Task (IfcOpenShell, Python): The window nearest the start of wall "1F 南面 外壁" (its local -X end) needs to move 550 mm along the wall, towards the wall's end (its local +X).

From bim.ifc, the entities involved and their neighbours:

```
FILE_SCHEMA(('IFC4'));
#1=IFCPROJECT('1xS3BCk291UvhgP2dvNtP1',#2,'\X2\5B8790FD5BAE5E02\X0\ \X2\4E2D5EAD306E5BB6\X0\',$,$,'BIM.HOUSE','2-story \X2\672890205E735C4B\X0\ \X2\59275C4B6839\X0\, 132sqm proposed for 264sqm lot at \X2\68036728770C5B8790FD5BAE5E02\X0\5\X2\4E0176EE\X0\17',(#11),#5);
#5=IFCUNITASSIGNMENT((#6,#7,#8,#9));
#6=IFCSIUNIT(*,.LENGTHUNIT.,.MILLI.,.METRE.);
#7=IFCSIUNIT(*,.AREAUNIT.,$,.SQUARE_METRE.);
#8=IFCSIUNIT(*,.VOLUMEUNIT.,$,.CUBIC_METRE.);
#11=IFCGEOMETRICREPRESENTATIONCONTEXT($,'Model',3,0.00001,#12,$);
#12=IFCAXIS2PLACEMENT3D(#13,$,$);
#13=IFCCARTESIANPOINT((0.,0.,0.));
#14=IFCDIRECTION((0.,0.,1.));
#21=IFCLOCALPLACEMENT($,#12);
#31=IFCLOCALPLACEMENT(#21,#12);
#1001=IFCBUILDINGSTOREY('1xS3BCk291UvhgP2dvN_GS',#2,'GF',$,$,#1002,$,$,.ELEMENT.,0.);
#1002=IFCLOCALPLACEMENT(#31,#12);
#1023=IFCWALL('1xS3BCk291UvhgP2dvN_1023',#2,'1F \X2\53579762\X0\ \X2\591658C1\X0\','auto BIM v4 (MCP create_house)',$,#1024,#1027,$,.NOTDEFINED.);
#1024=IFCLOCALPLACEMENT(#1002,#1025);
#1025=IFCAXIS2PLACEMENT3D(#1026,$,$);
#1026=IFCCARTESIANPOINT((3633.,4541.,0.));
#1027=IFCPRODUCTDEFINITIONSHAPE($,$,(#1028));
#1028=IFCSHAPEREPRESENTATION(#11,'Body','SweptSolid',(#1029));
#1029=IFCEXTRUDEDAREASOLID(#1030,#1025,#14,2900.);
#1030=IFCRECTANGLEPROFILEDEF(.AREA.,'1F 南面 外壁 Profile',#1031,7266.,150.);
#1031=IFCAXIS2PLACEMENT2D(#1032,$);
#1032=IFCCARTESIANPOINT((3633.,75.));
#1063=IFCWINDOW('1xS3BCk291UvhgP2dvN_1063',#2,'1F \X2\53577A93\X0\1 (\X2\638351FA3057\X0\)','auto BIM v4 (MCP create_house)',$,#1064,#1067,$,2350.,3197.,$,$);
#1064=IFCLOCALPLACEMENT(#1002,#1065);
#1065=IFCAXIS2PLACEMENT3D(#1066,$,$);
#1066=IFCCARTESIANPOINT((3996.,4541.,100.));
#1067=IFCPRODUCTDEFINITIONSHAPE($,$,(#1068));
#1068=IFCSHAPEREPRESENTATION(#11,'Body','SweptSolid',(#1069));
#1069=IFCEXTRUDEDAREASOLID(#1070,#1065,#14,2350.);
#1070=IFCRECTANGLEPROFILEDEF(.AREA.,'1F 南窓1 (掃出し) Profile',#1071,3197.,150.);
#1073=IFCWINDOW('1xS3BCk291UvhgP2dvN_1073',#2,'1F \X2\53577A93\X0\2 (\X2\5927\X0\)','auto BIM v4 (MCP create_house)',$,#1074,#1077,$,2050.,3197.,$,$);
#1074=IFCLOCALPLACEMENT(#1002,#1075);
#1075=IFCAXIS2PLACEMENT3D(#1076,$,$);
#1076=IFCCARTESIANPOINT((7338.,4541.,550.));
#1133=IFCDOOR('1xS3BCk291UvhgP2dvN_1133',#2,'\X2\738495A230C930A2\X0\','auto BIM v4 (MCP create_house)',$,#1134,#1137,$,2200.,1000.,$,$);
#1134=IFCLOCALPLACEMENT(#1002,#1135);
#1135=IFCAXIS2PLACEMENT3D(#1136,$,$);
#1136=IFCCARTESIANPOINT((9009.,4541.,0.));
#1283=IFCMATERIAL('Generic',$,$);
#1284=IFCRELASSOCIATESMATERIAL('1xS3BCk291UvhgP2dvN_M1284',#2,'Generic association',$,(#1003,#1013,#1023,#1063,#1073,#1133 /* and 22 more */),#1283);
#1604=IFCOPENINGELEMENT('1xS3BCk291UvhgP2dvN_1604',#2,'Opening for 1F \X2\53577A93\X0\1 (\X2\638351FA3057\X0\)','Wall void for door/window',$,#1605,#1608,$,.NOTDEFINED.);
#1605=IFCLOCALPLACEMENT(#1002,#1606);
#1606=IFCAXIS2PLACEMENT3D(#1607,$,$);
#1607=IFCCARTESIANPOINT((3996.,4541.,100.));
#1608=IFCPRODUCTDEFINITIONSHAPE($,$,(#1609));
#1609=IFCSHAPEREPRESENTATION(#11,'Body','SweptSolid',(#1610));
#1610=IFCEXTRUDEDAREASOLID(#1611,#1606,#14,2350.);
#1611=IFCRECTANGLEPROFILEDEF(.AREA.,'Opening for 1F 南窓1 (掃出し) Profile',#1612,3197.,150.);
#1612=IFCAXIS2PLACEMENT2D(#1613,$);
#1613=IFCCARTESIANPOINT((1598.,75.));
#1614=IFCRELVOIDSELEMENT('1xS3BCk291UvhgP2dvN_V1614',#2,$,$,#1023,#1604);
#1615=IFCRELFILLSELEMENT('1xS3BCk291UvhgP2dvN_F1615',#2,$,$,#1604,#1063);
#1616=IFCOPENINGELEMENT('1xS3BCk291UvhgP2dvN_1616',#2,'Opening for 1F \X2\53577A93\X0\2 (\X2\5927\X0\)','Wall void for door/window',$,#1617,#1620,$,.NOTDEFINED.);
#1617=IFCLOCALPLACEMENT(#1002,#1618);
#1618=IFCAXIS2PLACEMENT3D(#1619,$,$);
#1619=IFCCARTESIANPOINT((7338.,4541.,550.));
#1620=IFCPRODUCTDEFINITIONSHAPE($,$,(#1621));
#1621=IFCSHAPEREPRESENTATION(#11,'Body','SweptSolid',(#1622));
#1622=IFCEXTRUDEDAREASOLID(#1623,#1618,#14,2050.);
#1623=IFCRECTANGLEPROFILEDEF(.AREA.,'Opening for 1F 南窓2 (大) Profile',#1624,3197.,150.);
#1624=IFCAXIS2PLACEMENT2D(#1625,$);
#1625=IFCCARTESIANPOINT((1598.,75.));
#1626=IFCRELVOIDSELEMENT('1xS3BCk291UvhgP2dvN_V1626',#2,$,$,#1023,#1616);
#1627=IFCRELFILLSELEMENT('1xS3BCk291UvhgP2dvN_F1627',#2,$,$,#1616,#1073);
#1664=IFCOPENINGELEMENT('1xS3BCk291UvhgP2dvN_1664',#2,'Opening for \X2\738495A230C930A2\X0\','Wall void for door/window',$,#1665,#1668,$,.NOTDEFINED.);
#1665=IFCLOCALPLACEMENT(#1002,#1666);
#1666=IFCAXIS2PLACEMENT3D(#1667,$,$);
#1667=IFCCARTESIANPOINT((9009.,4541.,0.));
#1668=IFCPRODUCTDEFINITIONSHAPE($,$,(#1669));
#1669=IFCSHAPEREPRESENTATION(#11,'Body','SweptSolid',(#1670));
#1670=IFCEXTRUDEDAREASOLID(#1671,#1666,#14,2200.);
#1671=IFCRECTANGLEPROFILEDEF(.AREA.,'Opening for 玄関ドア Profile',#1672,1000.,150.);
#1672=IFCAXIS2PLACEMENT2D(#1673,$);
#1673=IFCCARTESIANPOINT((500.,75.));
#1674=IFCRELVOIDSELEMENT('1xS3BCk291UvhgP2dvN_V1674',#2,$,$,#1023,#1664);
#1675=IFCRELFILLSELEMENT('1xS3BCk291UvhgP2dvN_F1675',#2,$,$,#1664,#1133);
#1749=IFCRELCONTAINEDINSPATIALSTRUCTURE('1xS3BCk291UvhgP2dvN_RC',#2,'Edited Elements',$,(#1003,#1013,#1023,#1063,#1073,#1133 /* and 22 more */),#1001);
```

```python
import ifcopenshell
import ifcopenshell.api.geometry
import ifcopenshell.util.placement
import ifcopenshell.util.unit

model = ifcopenshell.open("bim.ifc")
unit_scale = ifcopenshell.util.unit.calculate_unit_scale(model)

window = model.by_guid("1xS3BCk291UvhgP2dvN_1063")
opening = window.FillsVoids[0].RelatingOpeningElement
wall = opening.VoidsElements[0].RelatingBuildingElement

wall_matrix = ifcopenshell.util.placement.get_local_placement(wall.ObjectPlacement)
shift = wall_matrix[:3, 0] * 0.55 / unit_scale
before = ifcopenshell.util.placement.get_local_placement(window.ObjectPlacement)[:3, 3].copy()

# The window is not placed relative to its opening, so move both.
for product in (opening, window):
    matrix = ifcopenshell.util.placement.get_local_placement(product.ObjectPlacement)
    matrix[:3, 3] += shift
    ifcopenshell.api.geometry.edit_object_placement(model, product=product, matrix=matrix, is_si=False)

after = ifcopenshell.util.placement.get_local_placement(window.ObjectPlacement)[:3, 3]
print("window moved by", (after - before).round(3) + 0.0)

model.write("bim_v2.ifc")
```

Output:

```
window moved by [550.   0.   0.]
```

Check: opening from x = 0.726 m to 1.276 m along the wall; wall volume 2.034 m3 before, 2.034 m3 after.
